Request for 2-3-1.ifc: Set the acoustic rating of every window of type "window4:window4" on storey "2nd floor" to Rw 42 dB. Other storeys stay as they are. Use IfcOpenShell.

First a look at what the model holds.

```python
import ifcopenshell
import ifcopenshell.util.element

model = ifcopenshell.open("2-3-1.ifc")
print(model.schema)
storey = next(s for s in model.by_type("IfcBuildingStorey") if s.Name == "2nd floor")
windows = [e for e in ifcopenshell.util.element.get_decomposition(storey) if e.is_a("IfcWindow")]
seen = {}
for e in windows:
    element_type = ifcopenshell.util.element.get_type(e)
    key = (element_type.Name if element_type != e and element_type else None, ifcopenshell.util.element.get_pset(e, "Pset_WindowCommon", "AcousticRating"))
    seen[key] = seen.get(key, 0) + 1
for (name, value), count in sorted(seen.items(), key=str):
    print(count, "x", name, "|", value)
```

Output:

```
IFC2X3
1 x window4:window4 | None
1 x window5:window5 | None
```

```python
import ifcopenshell
import ifcopenshell.api.pset
import ifcopenshell.util.element

model = ifcopenshell.open("2-3-1.ifc")

storey = next(s for s in model.by_type("IfcBuildingStorey") if s.Name == "2nd floor")
windows = [e for e in ifcopenshell.util.element.get_decomposition(storey) if e.is_a("IfcWindow")]

count = 0
for e in windows:
    element_type = ifcopenshell.util.element.get_type(e)
    if element_type in (None, e) or element_type.Name != "window4:window4":
        continue
    # add_pset returns the element's existing set when there is one.
    pset = ifcopenshell.api.pset.add_pset(model, product=e, name="Pset_WindowCommon")
    ifcopenshell.api.pset.edit_pset(model, pset=pset, properties={"AcousticRating": "Rw 42 dB"})
    count += 1

print(count, "windows updated")

model.write("2-3-1_v2.ifc")
```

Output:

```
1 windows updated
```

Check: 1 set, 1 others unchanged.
